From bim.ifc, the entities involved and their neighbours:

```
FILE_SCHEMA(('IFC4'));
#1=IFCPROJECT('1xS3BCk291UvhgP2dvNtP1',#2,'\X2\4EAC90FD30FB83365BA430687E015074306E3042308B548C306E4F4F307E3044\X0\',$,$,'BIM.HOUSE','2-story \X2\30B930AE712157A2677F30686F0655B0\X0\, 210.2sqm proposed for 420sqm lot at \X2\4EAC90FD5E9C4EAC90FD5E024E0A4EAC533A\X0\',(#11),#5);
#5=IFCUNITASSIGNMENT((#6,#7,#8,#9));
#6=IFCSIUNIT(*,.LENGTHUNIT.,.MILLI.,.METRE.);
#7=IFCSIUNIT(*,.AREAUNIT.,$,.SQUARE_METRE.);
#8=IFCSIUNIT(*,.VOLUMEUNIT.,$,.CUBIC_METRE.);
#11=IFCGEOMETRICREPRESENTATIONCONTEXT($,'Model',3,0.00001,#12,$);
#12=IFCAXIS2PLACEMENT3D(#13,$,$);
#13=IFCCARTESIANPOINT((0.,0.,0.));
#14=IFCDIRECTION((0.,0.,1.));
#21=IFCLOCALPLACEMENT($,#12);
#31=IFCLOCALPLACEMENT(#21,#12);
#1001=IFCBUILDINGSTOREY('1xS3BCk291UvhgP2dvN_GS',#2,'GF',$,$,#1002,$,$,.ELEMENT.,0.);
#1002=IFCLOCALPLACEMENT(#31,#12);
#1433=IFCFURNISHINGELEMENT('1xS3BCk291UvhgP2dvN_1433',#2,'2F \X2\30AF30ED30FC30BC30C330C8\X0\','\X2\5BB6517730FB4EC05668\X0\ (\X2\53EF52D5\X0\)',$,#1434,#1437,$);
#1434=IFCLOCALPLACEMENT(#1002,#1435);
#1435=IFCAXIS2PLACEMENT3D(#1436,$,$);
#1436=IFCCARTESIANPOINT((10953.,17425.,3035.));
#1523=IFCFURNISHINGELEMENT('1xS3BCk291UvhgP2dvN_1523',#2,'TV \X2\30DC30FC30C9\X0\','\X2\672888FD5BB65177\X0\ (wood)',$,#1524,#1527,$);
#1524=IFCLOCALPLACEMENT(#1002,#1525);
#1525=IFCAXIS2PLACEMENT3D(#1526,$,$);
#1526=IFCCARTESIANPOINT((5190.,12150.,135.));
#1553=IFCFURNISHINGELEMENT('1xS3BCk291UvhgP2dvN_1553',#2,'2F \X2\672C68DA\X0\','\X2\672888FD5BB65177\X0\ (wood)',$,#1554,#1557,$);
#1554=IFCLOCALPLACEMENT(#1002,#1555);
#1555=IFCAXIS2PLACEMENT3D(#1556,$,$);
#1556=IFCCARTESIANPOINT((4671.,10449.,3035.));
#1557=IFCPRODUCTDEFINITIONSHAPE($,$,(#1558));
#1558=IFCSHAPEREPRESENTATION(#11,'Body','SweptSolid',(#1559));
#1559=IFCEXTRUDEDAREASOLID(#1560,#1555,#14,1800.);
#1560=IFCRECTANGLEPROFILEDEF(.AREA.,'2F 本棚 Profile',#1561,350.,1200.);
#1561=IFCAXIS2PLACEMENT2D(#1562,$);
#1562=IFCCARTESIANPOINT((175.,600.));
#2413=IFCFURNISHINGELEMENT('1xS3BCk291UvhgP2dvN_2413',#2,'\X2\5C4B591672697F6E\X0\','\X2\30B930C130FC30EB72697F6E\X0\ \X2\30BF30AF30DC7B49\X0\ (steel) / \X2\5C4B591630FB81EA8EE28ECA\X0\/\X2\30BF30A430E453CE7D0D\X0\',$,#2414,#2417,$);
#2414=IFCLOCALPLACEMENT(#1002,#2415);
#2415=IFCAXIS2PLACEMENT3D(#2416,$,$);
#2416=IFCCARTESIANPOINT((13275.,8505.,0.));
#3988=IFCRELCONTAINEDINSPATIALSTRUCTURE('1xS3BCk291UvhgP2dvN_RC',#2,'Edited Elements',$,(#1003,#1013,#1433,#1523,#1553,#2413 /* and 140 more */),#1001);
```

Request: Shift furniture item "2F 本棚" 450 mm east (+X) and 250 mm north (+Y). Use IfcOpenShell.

```python
import ifcopenshell
import ifcopenshell.api.geometry
import ifcopenshell.util.placement

model = ifcopenshell.open("bim.ifc")

item = model.by_id(1553)
matrix = ifcopenshell.util.placement.get_local_placement(item.ObjectPlacement)
matrix[0, 3] += 450.0
matrix[1, 3] += 250.0
ifcopenshell.api.geometry.edit_object_placement(model, product=item, matrix=matrix, is_si=False)

print(ifcopenshell.util.placement.get_local_placement(item.ObjectPlacement).round(3) + 0.0)

model.write("bim_rev.ifc")
```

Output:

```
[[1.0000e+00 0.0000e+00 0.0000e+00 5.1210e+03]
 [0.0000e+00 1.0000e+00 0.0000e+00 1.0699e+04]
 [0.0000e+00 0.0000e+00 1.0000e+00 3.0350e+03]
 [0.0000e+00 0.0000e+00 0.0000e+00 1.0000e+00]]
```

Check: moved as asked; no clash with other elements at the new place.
